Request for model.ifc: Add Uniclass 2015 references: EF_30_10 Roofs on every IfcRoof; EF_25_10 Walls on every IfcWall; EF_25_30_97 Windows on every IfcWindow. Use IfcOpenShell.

First a look at what the model holds.

```python
import ifcopenshell

model = ifcopenshell.open("model.ifc")
print(model.schema)
print("classifications:", [c.Name for c in model.by_type("IfcClassification")])
for ifc_class in ("IfcDoor", "IfcRoof", "IfcStair", "IfcWall", "IfcWindow"):
    print(ifc_class, len(model.by_type(ifc_class)))
```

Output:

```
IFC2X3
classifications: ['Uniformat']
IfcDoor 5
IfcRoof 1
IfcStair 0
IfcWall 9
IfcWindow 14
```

```python
import ifcopenshell
import ifcopenshell.api.classification

model = ifcopenshell.open("model.ifc")

# IFC2X3 requires Source and Edition and has no link from the project to the system.
system = model.create_entity("IfcClassification", Source="NBS", Edition="2015", Name="Uniclass 2015")

codes = {
    "IfcRoof": ("EF_30_10", "Roofs"),
    "IfcWall": ("EF_25_10", "Walls"),
    "IfcWindow": ("EF_25_30_97", "Windows"),
}
for ifc_class, (code, name) in codes.items():
    products = model.by_type(ifc_class)
    ifcopenshell.api.classification.add_reference(
        model, products=products, classification=system, identification=code, name=name
    )
    print(code, len(products))

model.write("model_edited.ifc")
```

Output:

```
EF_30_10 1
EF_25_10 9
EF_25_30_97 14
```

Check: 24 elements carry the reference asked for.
